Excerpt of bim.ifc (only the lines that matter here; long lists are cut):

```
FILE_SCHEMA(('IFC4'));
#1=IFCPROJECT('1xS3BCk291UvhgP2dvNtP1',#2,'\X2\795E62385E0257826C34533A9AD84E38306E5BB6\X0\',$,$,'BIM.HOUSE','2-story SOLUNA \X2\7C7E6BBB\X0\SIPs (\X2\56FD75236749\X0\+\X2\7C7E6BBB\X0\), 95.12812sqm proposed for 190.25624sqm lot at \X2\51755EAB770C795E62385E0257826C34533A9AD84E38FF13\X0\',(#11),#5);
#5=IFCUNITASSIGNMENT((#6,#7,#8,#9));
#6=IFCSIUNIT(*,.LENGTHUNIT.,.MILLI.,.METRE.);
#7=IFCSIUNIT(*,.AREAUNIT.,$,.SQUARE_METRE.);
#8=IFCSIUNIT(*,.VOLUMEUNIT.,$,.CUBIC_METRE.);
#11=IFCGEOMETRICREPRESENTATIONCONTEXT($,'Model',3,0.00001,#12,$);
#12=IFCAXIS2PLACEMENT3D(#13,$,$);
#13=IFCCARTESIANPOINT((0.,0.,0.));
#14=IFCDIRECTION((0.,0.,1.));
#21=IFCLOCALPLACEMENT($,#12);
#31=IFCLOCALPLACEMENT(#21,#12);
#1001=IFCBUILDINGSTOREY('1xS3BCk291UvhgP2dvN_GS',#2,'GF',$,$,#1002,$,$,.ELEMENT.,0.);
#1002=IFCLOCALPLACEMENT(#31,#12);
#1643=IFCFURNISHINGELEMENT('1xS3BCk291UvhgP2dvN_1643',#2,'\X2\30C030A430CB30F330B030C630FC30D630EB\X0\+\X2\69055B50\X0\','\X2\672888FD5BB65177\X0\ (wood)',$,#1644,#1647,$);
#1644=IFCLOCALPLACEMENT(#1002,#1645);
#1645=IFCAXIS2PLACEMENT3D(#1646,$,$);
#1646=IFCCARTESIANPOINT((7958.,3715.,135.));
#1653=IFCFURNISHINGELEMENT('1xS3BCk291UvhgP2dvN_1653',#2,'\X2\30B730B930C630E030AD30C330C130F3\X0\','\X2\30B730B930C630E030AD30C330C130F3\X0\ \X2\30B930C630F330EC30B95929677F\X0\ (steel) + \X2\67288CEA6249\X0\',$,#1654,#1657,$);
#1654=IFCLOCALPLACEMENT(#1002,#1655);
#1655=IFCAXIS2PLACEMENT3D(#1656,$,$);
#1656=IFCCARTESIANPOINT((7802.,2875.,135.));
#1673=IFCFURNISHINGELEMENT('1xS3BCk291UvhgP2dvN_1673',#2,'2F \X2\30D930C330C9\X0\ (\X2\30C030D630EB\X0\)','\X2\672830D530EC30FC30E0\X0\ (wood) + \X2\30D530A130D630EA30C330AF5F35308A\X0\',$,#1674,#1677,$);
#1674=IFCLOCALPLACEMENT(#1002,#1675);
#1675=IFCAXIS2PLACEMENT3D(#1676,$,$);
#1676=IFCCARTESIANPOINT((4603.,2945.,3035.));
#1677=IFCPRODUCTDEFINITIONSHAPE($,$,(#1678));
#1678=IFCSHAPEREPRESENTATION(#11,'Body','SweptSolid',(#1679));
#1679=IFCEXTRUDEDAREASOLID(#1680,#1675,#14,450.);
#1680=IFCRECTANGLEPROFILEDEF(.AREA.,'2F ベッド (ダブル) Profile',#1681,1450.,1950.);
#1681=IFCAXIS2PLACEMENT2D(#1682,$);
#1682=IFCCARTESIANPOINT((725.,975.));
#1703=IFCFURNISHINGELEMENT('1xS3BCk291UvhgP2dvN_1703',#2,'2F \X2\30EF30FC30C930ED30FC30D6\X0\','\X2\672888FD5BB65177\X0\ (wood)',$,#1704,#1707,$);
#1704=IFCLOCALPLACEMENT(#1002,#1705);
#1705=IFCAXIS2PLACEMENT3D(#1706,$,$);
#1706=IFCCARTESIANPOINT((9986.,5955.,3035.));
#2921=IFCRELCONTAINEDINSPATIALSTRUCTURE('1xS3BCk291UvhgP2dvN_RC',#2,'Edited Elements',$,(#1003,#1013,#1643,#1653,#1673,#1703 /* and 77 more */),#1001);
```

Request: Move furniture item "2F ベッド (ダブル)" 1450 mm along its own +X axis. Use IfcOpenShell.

```python
import ifcopenshell
import ifcopenshell.api.geometry
import ifcopenshell.util.placement

model = ifcopenshell.open("bim.ifc")

item = model.by_guid("1xS3BCk291UvhgP2dvN_1673")
matrix = ifcopenshell.util.placement.get_local_placement(item.ObjectPlacement)
matrix[:3, 3] += matrix[:3, 0] * 1450.0
ifcopenshell.api.geometry.edit_object_placement(model, product=item, matrix=matrix, is_si=False)

print(ifcopenshell.util.placement.get_local_placement(item.ObjectPlacement).round(3) + 0.0)

model.write("bim_rev.ifc")
```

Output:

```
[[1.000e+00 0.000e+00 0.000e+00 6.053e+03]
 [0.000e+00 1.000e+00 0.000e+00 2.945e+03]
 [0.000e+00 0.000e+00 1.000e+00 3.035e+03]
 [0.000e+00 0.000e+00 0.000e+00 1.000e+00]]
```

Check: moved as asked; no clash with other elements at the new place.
